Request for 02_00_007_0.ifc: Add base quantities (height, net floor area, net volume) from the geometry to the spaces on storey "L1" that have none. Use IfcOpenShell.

First a look at what the model holds.

```python
import ifcopenshell
import ifcopenshell.util.element
import ifcopenshell.util.unit

model = ifcopenshell.open("02_00_007_0.ifc")
print(model.schema)
for unit_type in ("LENGTHUNIT", "AREAUNIT", "VOLUMEUNIT"):
    print(unit_type, ifcopenshell.util.unit.calculate_unit_scale(model, unit_type))
storey = next(s for s in model.by_type("IfcBuildingStorey") if s.Name == "L1")
spaces = [e for e in ifcopenshell.util.element.get_decomposition(storey) if e.is_a("IfcSpace")]
for e in sorted(spaces, key=lambda e: e.id()):
    print(e.id(), e.is_a(), e.Name, list(ifcopenshell.util.element.get_psets(e, qtos_only=True)), sep=" | ")
```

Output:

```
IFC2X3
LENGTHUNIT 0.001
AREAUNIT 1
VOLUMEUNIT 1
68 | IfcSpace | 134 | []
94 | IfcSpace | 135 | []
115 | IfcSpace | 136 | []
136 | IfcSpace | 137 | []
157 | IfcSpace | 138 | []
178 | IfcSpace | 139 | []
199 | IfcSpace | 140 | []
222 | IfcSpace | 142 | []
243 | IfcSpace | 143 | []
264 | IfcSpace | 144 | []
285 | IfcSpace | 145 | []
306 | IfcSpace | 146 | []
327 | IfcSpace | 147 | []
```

```python
import ifcopenshell
import ifcopenshell.api.pset
import ifcopenshell.geom
import ifcopenshell.util.element
import ifcopenshell.util.shape
import ifcopenshell.util.unit

model = ifcopenshell.open("02_00_007_0.ifc")
unit_scale = ifcopenshell.util.unit.calculate_unit_scale(model)
area_scale = ifcopenshell.util.unit.calculate_unit_scale(model, "AREAUNIT")
volume_scale = ifcopenshell.util.unit.calculate_unit_scale(model, "VOLUMEUNIT")
settings = ifcopenshell.geom.settings()

storey = next(s for s in model.by_type("IfcBuildingStorey") if s.Name == "L1")
spaces = [e for e in ifcopenshell.util.element.get_decomposition(storey) if e.is_a("IfcSpace")]

for e in sorted(spaces, key=lambda e: e.id()):
    if ifcopenshell.util.element.get_psets(e, qtos_only=True, should_inherit=False):
        continue
    # Geometry comes back in metres, in the element's own axes.
    shape = ifcopenshell.geom.create_shape(settings, e)
    values = {
        "Height": ifcopenshell.util.shape.get_z(shape.geometry) / unit_scale,
        "NetFloorArea": ifcopenshell.util.shape.get_footprint_area(shape.geometry) / area_scale,
        "NetVolume": ifcopenshell.util.shape.get_volume(shape.geometry) / volume_scale,
    }
    qto = ifcopenshell.api.pset.add_qto(model, product=e, name="BaseQuantities")
    ifcopenshell.api.pset.edit_qto(model, qto=qto, properties=values)
    print(e.id(), {k: round(v, 3) for k, v in values.items()})

model.write("02_00_007_0-out.ifc")
```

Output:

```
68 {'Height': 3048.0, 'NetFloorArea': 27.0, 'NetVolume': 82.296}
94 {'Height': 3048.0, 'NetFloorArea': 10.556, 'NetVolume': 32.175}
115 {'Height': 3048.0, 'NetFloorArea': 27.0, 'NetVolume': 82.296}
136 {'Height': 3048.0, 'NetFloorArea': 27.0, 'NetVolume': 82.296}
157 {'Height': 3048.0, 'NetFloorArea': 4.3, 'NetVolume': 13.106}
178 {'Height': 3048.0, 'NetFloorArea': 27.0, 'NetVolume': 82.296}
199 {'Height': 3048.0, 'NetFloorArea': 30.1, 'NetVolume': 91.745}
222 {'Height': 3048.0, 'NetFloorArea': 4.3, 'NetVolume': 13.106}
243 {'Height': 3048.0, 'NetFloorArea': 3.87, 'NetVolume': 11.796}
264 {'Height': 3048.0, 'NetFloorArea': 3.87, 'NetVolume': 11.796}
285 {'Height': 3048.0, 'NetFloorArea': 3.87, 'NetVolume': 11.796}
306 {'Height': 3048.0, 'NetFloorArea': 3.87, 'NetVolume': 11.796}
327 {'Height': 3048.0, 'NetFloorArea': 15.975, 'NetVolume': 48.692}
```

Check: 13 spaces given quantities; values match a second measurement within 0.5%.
